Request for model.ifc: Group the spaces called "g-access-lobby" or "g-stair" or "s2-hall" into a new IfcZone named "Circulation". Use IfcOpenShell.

First a look at what the model holds.

```python
import ifcopenshell

model = ifcopenshell.open("model.ifc")
print(model.schema)
seen = {}
for space in model.by_type("IfcSpace"):
    seen[space.LongName] = seen.get(space.LongName, 0) + 1
for name, count in sorted(seen.items(), key=str):
    print(count, "x", name)
print("zones:", [z.Name for z in model.by_type("IfcZone")][:20])
```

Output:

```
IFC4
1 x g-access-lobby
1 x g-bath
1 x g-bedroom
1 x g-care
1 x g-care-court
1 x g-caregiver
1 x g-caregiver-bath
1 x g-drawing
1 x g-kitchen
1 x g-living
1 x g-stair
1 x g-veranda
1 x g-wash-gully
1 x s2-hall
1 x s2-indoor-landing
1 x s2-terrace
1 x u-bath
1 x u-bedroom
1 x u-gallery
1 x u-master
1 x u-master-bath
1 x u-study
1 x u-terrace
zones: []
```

```python
import ifcopenshell
import ifcopenshell.api.group
import ifcopenshell.api.root

model = ifcopenshell.open("model.ifc")

names = {"g-access-lobby", "g-stair", "s2-hall"}
spaces = [s for s in model.by_type("IfcSpace") if s.LongName in names]

zone = ifcopenshell.api.root.create_entity(model, ifc_class="IfcZone", name="Circulation")
ifcopenshell.api.group.assign_group(model, products=spaces, group=zone)
print(len(spaces), "spaces in", zone.Name)

model.write("model_updated.ifc")
```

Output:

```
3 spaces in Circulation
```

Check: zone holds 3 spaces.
